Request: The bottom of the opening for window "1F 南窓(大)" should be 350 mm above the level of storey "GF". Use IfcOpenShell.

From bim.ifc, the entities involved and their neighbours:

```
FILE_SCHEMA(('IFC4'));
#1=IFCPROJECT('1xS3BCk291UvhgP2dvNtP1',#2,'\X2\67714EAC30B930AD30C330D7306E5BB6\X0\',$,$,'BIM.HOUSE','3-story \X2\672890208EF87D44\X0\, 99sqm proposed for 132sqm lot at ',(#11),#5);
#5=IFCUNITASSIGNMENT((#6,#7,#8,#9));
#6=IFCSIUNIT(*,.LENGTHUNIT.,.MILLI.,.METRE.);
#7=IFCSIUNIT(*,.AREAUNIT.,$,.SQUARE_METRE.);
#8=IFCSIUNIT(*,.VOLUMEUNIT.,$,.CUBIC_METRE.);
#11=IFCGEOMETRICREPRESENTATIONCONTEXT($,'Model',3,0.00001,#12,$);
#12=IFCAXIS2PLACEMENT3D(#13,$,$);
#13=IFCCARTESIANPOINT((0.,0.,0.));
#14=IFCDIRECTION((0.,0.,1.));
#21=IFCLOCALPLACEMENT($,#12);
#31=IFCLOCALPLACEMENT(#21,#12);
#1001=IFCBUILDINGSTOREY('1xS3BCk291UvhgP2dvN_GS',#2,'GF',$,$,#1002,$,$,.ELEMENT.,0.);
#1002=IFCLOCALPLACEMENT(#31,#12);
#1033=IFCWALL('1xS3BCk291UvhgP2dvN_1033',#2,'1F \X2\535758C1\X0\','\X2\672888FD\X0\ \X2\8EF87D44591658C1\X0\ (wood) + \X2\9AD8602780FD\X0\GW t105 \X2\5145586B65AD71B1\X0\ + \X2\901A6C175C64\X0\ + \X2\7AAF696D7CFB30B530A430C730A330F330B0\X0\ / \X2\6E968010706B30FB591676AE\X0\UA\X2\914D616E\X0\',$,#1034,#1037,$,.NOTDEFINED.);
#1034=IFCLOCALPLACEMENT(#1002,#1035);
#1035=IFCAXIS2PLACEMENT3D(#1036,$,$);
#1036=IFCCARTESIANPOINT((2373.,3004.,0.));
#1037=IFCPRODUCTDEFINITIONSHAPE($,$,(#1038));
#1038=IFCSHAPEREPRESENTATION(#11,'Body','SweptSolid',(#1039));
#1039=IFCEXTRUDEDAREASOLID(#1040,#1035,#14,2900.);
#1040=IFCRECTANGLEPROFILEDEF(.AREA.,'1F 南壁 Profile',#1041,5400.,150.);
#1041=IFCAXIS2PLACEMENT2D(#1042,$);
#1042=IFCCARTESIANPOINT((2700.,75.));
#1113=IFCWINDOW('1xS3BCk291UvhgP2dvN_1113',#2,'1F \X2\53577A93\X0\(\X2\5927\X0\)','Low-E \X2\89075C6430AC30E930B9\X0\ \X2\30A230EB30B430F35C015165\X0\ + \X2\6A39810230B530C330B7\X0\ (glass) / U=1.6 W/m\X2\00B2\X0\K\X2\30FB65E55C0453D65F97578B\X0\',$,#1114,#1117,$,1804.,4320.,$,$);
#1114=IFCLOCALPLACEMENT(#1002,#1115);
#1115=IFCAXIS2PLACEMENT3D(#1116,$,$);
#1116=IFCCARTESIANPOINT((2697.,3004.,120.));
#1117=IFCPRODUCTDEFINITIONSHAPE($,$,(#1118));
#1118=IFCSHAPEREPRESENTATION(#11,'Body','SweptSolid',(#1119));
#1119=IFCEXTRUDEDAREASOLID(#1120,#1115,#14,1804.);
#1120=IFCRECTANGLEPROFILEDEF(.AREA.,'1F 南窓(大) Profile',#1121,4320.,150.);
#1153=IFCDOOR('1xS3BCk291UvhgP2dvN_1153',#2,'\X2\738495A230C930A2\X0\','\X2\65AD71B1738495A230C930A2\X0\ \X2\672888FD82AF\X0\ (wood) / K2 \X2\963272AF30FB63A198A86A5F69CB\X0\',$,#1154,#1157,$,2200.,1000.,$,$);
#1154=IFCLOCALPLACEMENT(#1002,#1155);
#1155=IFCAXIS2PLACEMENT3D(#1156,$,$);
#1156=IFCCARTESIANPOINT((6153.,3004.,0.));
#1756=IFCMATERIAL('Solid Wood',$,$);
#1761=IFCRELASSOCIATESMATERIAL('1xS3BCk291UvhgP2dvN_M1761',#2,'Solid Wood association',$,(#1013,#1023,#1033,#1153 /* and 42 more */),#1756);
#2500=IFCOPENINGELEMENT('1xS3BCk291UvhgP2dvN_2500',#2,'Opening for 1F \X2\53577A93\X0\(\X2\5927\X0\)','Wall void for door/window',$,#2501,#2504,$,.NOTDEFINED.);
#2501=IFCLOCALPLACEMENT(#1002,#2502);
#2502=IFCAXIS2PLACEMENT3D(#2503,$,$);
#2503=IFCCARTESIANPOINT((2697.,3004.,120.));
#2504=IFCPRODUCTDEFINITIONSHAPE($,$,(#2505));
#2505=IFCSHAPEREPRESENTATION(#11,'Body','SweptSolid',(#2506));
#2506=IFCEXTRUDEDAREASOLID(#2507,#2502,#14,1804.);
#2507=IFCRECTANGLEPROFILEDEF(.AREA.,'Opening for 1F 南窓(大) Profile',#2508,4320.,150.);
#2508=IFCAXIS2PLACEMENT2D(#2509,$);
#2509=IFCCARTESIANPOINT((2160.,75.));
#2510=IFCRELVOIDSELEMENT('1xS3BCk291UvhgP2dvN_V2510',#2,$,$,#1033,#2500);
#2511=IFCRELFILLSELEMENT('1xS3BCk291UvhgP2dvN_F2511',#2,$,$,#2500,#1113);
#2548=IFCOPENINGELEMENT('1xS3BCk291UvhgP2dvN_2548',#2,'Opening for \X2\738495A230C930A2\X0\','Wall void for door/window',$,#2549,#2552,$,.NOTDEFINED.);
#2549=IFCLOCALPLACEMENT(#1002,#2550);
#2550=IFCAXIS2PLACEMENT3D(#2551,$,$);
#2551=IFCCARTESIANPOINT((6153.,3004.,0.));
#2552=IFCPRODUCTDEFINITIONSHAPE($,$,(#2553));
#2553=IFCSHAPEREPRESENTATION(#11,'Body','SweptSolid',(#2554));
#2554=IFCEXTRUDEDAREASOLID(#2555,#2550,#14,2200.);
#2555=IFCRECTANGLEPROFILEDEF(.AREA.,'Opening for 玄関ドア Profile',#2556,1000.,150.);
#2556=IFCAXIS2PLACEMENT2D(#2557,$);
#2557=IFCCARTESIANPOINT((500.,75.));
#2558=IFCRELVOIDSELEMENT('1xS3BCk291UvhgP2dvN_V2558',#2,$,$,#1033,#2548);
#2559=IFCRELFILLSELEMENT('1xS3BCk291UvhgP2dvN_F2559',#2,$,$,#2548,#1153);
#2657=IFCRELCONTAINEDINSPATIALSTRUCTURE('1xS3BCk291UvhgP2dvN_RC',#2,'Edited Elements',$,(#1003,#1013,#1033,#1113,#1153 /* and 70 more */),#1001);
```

```python
import numpy as np
import ifcopenshell
import ifcopenshell.api.geometry
import ifcopenshell.geom
import ifcopenshell.util.element
import ifcopenshell.util.placement
import ifcopenshell.util.shape
import ifcopenshell.util.unit

model = ifcopenshell.open("bim.ifc")
unit_scale = ifcopenshell.util.unit.calculate_unit_scale(model)

window = model.by_guid("1xS3BCk291UvhgP2dvN_1113")
opening = window.FillsVoids[0].RelatingOpeningElement
storey = ifcopenshell.util.element.get_container(window, ifc_class="IfcBuildingStorey")
level = ifcopenshell.util.placement.get_local_placement(storey.ObjectPlacement)[2, 3]

# The opening's origin need not be at the sill, so measure its lowest point.
shape = ifcopenshell.geom.create_shape(ifcopenshell.geom.settings(), opening)
bottom = ifcopenshell.util.shape.get_shape_bottom_elevation(shape, shape.geometry) / unit_scale
dz = level + 0.35 / unit_scale - bottom

shift = np.array([0.0, 0.0, dz])
# The window is not placed relative to its opening, so move both.
for product in (opening, window):
    matrix = ifcopenshell.util.placement.get_local_placement(product.ObjectPlacement)
    matrix[:3, 3] += shift
    ifcopenshell.api.geometry.edit_object_placement(model, product=product, matrix=matrix, is_si=False)

print(f"moved by {dz * unit_scale:+.3f} m")

model.write("bim_rev.ifc")
```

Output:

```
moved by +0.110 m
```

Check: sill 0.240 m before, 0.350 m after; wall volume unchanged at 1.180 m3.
